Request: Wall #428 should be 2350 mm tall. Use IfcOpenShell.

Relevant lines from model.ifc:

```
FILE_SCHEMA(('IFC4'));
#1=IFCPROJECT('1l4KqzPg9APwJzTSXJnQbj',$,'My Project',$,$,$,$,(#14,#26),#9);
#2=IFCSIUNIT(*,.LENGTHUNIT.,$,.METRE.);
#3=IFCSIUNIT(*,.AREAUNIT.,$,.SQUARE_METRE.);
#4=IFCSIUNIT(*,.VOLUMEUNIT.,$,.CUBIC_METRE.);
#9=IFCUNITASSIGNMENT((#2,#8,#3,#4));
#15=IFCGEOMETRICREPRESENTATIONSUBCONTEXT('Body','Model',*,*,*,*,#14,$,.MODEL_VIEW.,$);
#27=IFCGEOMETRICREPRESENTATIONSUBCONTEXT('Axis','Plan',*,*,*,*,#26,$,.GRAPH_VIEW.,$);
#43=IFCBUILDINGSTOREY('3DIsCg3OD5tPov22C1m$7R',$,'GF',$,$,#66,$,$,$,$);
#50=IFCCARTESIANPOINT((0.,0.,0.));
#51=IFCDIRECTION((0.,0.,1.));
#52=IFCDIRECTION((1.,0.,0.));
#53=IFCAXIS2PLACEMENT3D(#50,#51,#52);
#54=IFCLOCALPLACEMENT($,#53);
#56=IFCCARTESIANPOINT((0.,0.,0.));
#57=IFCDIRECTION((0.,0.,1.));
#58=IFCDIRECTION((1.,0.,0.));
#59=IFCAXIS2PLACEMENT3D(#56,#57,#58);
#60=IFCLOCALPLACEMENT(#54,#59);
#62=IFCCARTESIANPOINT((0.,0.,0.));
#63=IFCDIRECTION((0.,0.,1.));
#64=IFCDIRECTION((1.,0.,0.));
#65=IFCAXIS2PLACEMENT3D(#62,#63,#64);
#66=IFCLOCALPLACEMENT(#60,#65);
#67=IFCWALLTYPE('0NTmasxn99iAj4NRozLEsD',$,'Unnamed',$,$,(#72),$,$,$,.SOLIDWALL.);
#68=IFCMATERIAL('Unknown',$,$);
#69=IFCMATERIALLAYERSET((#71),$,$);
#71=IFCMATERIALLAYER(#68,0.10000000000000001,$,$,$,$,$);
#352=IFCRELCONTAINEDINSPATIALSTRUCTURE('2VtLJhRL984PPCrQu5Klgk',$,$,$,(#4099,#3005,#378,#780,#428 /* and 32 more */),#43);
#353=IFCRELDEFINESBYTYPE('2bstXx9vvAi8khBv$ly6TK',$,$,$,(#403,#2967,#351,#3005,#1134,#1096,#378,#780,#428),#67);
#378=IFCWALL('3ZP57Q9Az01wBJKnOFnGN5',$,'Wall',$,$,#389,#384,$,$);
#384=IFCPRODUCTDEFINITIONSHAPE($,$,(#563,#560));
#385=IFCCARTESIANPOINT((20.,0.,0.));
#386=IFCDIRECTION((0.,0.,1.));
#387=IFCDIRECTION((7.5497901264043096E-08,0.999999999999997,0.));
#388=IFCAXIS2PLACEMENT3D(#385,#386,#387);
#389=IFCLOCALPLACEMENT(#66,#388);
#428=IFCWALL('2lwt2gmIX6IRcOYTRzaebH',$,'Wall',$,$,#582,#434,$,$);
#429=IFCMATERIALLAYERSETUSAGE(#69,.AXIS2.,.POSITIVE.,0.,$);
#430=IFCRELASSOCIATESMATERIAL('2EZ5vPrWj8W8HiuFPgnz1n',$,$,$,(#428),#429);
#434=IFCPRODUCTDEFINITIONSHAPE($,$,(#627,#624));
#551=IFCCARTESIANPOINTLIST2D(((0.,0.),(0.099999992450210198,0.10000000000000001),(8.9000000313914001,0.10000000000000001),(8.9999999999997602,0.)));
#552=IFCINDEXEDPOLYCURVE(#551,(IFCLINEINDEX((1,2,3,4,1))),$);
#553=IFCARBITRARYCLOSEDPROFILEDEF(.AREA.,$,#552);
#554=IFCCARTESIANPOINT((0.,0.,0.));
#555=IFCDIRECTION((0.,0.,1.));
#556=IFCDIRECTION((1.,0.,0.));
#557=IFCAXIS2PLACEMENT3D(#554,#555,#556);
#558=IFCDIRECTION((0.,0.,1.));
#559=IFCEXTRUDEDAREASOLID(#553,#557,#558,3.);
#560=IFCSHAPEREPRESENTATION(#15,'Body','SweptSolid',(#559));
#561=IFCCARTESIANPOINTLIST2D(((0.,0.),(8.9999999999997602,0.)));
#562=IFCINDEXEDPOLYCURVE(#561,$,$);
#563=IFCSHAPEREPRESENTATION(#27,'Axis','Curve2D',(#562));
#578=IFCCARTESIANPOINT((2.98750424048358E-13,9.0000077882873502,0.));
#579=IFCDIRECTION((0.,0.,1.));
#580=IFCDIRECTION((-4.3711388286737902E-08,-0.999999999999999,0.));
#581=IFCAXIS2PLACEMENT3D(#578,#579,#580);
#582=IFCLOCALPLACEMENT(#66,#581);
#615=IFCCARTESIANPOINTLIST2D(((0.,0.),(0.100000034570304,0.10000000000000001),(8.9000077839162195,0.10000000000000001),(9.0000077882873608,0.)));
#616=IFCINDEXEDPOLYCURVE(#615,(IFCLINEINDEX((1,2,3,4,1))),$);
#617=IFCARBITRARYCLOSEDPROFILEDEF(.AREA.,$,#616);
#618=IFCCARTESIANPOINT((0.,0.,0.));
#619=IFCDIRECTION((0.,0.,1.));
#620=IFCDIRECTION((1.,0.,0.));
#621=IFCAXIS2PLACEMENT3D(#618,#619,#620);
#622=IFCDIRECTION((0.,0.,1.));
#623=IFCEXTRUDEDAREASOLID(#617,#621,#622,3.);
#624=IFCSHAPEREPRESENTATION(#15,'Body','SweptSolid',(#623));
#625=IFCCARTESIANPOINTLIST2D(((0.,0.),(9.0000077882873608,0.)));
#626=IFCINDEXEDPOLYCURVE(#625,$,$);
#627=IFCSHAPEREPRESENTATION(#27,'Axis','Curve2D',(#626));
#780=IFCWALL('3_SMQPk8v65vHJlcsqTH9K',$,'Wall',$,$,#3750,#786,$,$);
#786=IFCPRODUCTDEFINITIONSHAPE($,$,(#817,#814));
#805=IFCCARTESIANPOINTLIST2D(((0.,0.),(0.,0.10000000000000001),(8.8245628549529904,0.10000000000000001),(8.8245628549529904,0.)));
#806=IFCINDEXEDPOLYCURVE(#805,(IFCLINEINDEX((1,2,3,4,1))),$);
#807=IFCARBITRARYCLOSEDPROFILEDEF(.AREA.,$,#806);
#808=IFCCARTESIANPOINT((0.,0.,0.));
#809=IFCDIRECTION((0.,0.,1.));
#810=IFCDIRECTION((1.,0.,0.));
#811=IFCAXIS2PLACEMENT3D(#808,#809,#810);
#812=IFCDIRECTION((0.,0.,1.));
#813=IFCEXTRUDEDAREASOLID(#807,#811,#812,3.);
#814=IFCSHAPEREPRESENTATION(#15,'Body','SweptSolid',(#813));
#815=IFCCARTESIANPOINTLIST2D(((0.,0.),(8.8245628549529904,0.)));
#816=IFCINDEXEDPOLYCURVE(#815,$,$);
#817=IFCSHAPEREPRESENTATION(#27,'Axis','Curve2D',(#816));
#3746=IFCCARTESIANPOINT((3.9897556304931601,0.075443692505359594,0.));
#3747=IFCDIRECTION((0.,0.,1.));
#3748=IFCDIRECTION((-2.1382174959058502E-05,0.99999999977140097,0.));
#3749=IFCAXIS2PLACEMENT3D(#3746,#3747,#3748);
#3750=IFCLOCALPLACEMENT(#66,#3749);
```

```python
import ifcopenshell
import ifcopenshell.geom
import ifcopenshell.util.representation
import ifcopenshell.util.shape
import ifcopenshell.util.unit

model = ifcopenshell.open("model.ifc")
unit_scale = ifcopenshell.util.unit.calculate_unit_scale(model)
settings = ifcopenshell.geom.settings()


def volume(element):
    """Net volume in cubic metres, openings subtracted."""
    shape = ifcopenshell.geom.create_shape(settings, element)
    return ifcopenshell.util.shape.get_volume(shape.geometry)


wall = model.by_guid("2lwt2gmIX6IRcOYTRzaebH")
before = volume(wall)

body = ifcopenshell.util.representation.get_representation(wall, "Model", "Body")
solid = body.Items[0]
old_height = solid.Depth
solid.Depth = 2.35 / unit_scale
after = volume(wall)

print(f"height {old_height:g} -> {solid.Depth:g}, volume {before:.3f} -> {after:.3f} m3")

model.write("model_v2.ifc")
```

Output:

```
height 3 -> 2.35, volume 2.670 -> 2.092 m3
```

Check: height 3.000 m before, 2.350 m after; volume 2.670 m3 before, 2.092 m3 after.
